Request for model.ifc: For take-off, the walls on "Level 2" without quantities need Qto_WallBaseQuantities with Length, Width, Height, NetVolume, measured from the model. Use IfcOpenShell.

First a look at what the model holds.

```python
import ifcopenshell
import ifcopenshell.util.element
import ifcopenshell.util.unit

model = ifcopenshell.open("model.ifc")
print(model.schema)
for unit_type in ("LENGTHUNIT", "AREAUNIT", "VOLUMEUNIT"):
    print(unit_type, ifcopenshell.util.unit.calculate_unit_scale(model, unit_type))
storey = next(s for s in model.by_type("IfcBuildingStorey") if s.Name == "Level 2")
walls = [e for e in ifcopenshell.util.element.get_decomposition(storey) if e.is_a("IfcWall")]
for e in sorted(walls, key=lambda e: e.id()):
    print(e.id(), e.is_a(), e.Name, list(ifcopenshell.util.element.get_psets(e, qtos_only=True)), sep=" | ")
```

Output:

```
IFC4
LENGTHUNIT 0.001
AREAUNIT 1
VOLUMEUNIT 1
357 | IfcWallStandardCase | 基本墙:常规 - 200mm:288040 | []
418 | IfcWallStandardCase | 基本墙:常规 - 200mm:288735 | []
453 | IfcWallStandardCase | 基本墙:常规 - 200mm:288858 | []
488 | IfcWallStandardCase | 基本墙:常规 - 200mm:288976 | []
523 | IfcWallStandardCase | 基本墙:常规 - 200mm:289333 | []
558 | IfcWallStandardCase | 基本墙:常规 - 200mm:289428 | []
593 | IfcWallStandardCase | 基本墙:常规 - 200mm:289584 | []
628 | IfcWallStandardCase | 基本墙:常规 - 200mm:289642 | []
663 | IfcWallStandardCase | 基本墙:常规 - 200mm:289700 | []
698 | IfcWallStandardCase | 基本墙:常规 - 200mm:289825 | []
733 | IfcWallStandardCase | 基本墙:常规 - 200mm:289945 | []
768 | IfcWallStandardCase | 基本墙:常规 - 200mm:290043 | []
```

```python
import ifcopenshell
import ifcopenshell.api.pset
import ifcopenshell.geom
import ifcopenshell.util.element
import ifcopenshell.util.shape
import ifcopenshell.util.unit

model = ifcopenshell.open("model.ifc")
unit_scale = ifcopenshell.util.unit.calculate_unit_scale(model)
volume_scale = ifcopenshell.util.unit.calculate_unit_scale(model, "VOLUMEUNIT")
settings = ifcopenshell.geom.settings()

storey = next(s for s in model.by_type("IfcBuildingStorey") if s.Name == "Level 2")
walls = [e for e in ifcopenshell.util.element.get_decomposition(storey) if e.is_a("IfcWall")]

for e in sorted(walls, key=lambda e: e.id()):
    if ifcopenshell.util.element.get_psets(e, qtos_only=True, should_inherit=False):
        continue
    # Geometry comes back in metres, in the element's own axes.
    shape = ifcopenshell.geom.create_shape(settings, e)
    values = {
        "Length": ifcopenshell.util.shape.get_x(shape.geometry) / unit_scale,
        "Width": ifcopenshell.util.shape.get_y(shape.geometry) / unit_scale,
        "Height": ifcopenshell.util.shape.get_z(shape.geometry) / unit_scale,
        "NetVolume": ifcopenshell.util.shape.get_volume(shape.geometry) / volume_scale,
    }
    qto = ifcopenshell.api.pset.add_qto(model, product=e, name="Qto_WallBaseQuantities")
    ifcopenshell.api.pset.edit_qto(model, qto=qto, properties=values)
    print(e.id(), {k: round(v, 3) for k, v in values.items()})

model.write("model_edited.ifc")
```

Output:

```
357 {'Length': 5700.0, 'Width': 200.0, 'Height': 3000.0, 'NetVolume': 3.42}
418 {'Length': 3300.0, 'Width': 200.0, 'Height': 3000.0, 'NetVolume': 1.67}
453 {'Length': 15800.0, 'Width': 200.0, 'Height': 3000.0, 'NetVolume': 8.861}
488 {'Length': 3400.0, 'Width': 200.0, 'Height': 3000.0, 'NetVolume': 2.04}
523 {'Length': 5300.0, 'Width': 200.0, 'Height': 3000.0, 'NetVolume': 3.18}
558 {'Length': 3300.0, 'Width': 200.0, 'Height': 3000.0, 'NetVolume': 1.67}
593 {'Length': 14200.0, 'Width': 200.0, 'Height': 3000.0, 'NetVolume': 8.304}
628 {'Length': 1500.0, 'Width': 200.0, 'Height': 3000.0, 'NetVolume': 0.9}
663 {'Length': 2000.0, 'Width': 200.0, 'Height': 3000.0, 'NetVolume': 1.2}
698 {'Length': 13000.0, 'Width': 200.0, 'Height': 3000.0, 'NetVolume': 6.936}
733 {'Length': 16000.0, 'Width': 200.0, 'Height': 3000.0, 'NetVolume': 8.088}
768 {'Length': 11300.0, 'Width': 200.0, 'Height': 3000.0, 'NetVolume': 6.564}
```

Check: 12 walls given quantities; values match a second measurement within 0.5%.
